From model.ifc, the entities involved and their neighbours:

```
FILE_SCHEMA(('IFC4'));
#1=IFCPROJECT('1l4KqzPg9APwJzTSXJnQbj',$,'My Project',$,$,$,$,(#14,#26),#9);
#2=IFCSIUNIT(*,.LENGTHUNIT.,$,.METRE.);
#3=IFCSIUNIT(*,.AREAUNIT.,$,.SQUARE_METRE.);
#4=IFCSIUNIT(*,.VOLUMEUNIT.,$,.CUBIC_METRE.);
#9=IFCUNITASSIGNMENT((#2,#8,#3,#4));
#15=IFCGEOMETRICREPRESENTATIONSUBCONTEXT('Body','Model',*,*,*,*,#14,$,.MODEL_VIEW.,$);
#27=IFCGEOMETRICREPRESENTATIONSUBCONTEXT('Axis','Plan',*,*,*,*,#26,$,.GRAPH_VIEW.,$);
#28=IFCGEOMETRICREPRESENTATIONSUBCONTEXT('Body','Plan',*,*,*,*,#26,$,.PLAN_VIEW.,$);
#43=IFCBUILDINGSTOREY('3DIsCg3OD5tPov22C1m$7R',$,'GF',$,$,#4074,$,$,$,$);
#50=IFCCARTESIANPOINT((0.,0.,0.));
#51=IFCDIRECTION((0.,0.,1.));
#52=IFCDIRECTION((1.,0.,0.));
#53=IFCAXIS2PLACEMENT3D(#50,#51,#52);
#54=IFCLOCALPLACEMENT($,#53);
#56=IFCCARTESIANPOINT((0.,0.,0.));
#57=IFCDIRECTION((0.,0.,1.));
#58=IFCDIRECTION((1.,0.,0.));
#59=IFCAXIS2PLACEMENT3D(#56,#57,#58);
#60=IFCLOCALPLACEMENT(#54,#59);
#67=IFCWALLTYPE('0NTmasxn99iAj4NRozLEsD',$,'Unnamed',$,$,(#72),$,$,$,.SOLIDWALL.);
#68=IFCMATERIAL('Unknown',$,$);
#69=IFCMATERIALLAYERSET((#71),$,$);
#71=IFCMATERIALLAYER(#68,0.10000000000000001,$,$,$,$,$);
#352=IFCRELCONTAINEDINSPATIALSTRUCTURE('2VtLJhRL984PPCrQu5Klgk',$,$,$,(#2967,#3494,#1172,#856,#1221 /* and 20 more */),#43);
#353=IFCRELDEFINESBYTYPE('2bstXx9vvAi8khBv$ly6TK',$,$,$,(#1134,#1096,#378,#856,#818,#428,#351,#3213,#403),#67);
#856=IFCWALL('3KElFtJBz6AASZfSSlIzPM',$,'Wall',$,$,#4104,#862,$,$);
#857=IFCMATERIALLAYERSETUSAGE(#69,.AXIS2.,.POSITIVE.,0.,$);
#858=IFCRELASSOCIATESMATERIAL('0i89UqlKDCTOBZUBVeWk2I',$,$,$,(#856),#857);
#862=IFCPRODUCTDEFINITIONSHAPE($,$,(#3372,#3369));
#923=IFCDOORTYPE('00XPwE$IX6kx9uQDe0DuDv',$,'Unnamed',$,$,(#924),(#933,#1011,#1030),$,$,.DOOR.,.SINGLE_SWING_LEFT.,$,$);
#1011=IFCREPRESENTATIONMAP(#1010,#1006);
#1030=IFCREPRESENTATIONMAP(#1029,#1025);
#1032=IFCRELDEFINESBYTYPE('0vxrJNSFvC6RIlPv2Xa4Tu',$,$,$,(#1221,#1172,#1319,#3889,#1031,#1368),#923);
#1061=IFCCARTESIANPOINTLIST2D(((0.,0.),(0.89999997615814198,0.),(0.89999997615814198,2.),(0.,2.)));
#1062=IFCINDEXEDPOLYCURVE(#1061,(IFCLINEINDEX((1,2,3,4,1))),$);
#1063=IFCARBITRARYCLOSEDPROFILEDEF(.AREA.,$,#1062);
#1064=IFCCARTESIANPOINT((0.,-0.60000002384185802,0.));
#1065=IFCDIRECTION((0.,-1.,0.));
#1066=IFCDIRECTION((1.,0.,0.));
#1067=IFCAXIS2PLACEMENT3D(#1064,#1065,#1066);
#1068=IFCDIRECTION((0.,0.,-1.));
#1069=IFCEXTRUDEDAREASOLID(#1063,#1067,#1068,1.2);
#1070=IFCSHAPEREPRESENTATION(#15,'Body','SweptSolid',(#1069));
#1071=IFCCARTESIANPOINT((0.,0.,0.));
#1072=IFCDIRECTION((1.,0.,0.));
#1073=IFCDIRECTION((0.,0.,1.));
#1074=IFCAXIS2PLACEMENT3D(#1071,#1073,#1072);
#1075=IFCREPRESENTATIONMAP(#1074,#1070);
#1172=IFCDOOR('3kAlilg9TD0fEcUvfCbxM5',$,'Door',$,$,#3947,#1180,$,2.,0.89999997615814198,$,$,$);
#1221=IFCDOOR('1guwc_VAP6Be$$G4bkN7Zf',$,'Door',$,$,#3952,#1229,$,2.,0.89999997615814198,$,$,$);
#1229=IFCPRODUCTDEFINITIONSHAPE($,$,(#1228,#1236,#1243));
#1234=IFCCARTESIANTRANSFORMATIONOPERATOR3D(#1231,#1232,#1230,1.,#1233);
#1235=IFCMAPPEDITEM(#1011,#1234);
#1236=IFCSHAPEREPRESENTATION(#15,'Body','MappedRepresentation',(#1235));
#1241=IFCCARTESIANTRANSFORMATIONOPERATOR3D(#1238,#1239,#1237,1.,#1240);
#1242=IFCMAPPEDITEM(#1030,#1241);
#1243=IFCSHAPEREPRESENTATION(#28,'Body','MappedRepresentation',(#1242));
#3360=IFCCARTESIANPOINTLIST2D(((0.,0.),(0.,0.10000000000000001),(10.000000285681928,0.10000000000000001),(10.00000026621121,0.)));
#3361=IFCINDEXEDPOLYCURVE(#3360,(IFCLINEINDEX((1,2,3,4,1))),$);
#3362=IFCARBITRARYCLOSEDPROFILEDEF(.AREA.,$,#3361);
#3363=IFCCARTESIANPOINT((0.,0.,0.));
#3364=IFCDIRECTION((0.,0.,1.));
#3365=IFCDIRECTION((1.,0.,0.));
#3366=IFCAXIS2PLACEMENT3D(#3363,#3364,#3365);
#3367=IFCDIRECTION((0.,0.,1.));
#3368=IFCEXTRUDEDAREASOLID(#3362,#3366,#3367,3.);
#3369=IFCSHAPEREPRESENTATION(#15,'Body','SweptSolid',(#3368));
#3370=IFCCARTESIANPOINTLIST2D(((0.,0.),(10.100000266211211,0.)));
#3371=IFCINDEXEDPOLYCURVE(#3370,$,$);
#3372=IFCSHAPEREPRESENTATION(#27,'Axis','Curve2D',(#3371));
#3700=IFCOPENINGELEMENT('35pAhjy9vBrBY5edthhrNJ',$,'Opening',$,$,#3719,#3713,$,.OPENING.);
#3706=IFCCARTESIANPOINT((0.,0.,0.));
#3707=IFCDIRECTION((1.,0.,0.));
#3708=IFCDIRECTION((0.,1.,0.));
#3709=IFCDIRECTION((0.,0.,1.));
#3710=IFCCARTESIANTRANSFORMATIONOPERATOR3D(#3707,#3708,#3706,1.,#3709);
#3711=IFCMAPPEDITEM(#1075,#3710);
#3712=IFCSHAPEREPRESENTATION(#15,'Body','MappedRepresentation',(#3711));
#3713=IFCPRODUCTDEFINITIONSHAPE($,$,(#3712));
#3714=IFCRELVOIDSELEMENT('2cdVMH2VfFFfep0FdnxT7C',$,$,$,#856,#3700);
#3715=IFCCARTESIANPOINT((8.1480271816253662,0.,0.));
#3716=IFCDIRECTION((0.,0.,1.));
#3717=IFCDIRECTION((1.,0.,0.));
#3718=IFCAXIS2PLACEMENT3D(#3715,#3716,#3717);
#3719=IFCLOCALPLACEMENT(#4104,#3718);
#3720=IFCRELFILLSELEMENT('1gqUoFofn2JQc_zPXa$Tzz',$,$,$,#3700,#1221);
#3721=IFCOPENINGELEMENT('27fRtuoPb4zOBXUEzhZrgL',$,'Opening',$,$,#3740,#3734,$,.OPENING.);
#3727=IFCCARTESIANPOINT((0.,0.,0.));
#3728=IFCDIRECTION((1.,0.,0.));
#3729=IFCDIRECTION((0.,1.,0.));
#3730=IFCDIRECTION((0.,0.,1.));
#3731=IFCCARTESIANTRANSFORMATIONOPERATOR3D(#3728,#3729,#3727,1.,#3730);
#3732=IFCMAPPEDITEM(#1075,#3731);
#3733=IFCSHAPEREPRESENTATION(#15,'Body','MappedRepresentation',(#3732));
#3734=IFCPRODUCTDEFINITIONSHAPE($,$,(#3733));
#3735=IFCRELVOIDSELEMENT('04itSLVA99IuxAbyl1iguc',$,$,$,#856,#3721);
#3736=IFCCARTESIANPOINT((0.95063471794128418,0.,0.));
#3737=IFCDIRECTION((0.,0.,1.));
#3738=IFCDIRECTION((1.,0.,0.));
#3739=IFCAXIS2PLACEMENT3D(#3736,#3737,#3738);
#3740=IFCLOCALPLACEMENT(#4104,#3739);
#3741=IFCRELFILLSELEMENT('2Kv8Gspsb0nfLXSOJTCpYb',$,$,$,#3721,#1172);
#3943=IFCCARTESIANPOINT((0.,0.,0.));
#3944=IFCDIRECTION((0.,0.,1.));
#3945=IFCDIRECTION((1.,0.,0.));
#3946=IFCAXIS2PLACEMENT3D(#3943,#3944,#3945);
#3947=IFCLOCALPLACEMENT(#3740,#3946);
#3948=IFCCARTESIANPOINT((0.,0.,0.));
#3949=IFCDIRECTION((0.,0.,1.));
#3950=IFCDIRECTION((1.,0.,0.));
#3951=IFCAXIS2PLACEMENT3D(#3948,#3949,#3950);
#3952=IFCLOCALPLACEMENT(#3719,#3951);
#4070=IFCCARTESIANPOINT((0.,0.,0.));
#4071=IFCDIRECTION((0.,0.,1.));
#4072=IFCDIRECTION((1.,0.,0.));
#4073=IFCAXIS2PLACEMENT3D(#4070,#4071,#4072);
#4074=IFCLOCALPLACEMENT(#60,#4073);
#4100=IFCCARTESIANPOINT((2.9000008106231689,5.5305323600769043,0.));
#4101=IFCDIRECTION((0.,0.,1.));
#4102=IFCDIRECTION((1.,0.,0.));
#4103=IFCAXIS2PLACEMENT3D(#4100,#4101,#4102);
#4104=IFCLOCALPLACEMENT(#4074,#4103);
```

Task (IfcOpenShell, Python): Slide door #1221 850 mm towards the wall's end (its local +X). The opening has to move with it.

```python
import ifcopenshell
import ifcopenshell.api.geometry
import ifcopenshell.util.placement
import ifcopenshell.util.unit

model = ifcopenshell.open("model.ifc")
unit_scale = ifcopenshell.util.unit.calculate_unit_scale(model)

door = model.by_guid("1guwc_VAP6Be$$G4bkN7Zf")
opening = door.FillsVoids[0].RelatingOpeningElement
wall = opening.VoidsElements[0].RelatingBuildingElement

wall_matrix = ifcopenshell.util.placement.get_local_placement(wall.ObjectPlacement)
shift = wall_matrix[:3, 0] * 0.85 / unit_scale
before = ifcopenshell.util.placement.get_local_placement(door.ObjectPlacement)[:3, 3].copy()

# The door is placed relative to its opening, so it follows when the opening moves.
matrix = ifcopenshell.util.placement.get_local_placement(opening.ObjectPlacement)
matrix[:3, 3] += shift
ifcopenshell.api.geometry.edit_object_placement(
    model, product=opening, matrix=matrix, is_si=False, should_transform_children=True
)

after = ifcopenshell.util.placement.get_local_placement(door.ObjectPlacement)[:3, 3]
print("door moved by", (after - before).round(3) + 0.0)

model.write("model-out.ifc")
```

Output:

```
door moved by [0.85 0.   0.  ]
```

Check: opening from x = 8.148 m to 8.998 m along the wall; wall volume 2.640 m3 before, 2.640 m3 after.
